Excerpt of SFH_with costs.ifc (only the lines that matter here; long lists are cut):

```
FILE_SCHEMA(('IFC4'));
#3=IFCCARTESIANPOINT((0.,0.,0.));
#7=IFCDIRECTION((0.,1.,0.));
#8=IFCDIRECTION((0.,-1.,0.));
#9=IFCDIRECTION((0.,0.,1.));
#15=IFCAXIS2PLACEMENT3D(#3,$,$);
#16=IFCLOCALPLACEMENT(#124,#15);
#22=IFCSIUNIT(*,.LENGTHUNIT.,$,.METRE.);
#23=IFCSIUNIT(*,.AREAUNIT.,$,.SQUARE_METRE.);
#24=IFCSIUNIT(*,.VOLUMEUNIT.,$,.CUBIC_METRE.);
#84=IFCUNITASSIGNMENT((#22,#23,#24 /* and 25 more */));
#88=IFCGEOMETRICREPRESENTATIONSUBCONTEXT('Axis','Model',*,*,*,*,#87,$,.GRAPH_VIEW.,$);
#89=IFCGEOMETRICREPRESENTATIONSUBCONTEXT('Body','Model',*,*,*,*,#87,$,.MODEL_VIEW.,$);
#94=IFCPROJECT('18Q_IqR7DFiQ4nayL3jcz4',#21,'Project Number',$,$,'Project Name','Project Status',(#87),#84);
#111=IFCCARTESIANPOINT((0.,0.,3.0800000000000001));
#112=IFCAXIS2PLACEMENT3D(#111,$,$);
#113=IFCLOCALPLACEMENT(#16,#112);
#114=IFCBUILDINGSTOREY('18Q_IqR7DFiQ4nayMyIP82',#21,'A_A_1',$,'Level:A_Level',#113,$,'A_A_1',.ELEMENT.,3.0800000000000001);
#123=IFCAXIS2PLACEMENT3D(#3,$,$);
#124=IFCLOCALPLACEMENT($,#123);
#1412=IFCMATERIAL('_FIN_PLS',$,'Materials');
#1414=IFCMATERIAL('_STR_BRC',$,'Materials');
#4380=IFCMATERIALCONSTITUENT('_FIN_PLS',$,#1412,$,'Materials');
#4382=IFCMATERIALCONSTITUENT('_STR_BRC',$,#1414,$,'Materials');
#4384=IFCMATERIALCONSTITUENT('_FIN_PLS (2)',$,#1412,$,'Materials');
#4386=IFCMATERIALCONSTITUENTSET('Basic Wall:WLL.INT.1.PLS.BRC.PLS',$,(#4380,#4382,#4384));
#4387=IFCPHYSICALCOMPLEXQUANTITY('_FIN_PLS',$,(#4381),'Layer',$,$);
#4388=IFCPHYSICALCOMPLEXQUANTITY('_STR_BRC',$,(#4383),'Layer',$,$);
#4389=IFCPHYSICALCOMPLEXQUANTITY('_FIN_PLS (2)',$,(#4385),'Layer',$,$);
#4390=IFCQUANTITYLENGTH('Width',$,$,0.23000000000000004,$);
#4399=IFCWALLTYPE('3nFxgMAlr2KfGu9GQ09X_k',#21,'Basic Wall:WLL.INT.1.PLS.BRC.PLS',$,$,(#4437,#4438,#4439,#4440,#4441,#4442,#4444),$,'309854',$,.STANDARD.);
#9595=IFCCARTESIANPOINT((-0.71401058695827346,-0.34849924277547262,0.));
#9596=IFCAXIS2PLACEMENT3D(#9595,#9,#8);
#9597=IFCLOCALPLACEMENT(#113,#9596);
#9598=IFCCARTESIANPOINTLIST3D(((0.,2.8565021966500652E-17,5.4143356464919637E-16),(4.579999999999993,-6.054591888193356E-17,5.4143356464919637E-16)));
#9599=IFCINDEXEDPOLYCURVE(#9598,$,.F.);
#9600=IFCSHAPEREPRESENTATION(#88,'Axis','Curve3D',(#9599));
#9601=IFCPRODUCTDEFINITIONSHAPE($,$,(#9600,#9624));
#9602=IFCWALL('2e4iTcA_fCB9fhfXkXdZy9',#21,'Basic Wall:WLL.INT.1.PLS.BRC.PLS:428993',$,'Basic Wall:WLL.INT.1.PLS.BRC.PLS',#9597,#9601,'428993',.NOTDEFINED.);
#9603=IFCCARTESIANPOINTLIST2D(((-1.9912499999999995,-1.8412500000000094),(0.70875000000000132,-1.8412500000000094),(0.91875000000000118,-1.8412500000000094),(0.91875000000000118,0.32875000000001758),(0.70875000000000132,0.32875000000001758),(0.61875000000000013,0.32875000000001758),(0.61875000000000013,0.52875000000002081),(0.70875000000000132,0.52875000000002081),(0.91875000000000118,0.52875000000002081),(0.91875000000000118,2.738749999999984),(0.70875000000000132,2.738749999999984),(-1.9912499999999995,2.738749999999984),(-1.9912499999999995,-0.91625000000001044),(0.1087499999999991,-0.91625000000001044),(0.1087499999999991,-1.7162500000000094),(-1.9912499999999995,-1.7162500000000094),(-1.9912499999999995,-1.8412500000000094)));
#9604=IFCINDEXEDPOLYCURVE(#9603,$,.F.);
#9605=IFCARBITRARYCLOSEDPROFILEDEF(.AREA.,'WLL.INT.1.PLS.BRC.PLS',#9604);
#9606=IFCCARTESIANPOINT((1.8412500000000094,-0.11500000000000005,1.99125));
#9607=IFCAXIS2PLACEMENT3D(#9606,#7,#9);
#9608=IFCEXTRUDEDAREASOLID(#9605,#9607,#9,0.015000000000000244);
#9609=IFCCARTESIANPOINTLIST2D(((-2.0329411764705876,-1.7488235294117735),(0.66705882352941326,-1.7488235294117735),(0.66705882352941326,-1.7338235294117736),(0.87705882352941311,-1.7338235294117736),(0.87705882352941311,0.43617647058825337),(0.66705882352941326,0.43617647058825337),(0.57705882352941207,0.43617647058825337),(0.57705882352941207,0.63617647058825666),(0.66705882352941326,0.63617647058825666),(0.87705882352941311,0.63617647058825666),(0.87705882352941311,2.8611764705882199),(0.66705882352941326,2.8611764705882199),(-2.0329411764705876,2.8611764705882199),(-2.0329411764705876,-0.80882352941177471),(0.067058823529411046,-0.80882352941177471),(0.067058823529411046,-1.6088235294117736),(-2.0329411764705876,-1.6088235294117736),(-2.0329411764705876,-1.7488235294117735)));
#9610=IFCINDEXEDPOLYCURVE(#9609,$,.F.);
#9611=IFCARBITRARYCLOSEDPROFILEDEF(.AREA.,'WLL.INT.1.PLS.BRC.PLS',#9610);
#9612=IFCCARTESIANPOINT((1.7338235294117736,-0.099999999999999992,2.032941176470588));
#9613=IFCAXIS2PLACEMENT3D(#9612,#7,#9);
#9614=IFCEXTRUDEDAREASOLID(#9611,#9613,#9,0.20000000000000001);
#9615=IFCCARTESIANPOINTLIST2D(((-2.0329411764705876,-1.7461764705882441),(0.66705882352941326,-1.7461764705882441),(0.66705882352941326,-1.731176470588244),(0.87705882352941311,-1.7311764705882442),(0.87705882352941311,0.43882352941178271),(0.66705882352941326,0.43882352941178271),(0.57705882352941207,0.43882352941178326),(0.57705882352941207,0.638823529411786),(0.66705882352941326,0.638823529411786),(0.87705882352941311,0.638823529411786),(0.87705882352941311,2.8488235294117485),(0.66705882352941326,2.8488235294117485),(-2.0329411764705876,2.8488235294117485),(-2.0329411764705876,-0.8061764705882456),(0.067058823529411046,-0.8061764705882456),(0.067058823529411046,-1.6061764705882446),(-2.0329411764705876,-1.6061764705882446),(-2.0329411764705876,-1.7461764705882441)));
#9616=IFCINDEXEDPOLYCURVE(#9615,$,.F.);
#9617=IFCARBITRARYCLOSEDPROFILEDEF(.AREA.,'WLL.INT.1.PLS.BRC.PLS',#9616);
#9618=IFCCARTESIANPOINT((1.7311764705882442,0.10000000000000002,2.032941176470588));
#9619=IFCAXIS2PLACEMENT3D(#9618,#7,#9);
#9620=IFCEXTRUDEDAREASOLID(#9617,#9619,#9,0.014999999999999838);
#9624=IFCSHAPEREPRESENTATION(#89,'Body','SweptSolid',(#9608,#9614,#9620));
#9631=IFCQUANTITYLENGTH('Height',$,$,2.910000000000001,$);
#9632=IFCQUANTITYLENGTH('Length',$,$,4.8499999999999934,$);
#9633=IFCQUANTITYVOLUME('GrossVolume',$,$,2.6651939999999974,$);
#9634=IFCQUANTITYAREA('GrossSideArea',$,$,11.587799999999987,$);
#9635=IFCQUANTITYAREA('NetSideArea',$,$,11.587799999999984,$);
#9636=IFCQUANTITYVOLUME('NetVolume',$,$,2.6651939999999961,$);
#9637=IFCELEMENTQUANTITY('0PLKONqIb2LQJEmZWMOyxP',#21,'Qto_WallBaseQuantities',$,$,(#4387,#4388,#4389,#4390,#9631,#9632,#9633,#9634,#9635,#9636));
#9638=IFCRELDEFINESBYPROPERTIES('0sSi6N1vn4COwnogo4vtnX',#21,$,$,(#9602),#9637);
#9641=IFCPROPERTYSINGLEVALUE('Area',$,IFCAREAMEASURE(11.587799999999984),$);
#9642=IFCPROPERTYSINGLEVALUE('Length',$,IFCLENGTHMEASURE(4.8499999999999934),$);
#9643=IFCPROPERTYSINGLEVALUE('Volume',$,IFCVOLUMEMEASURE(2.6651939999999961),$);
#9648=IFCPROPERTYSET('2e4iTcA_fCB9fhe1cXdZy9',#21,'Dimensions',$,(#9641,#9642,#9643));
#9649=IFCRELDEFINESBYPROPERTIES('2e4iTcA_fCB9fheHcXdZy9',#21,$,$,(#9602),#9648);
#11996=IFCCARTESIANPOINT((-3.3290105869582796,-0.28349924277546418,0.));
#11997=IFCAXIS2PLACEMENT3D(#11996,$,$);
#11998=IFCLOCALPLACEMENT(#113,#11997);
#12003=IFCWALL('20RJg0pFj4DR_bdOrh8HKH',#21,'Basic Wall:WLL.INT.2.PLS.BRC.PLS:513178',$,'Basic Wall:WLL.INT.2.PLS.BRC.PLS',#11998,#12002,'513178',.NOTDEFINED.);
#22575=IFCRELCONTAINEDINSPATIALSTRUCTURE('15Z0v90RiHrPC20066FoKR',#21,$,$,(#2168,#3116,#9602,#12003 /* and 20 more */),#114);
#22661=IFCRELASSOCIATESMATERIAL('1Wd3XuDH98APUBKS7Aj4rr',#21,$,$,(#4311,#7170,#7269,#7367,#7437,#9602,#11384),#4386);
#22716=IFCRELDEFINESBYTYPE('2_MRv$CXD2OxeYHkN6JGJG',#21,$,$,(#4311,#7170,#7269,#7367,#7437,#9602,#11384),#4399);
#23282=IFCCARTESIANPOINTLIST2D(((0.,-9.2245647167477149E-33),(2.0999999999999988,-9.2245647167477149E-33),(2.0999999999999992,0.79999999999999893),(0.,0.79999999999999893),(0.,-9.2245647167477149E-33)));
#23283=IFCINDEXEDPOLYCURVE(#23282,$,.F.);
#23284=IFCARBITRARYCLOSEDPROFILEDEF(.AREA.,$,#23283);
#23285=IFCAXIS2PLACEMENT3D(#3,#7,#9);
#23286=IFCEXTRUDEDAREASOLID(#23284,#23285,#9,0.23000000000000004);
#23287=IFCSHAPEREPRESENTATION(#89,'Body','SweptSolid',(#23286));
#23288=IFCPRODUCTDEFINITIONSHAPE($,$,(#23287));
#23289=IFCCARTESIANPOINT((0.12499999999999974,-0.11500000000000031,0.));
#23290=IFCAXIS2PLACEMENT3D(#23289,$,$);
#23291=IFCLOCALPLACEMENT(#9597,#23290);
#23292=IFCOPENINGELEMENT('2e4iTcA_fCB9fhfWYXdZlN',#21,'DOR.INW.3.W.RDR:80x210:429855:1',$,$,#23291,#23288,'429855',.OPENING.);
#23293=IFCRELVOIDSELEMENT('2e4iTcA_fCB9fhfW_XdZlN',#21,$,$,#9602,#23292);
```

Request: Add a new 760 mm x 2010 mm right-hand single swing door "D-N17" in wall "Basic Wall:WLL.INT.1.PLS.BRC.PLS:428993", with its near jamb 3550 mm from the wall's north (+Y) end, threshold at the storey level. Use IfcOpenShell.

```python
import numpy as np
import ifcopenshell
import ifcopenshell.api.feature
import ifcopenshell.api.geometry
import ifcopenshell.api.pset
import ifcopenshell.api.root
import ifcopenshell.api.spatial
import ifcopenshell.geom
import ifcopenshell.util.element
import ifcopenshell.util.placement
import ifcopenshell.util.representation
import ifcopenshell.util.shape
import ifcopenshell.util.unit

model = ifcopenshell.open("SFH_with costs.ifc")
unit_scale = ifcopenshell.util.unit.calculate_unit_scale(model)
area_scale = ifcopenshell.util.unit.calculate_unit_scale(model, "AREAUNIT")
volume_scale = ifcopenshell.util.unit.calculate_unit_scale(model, "VOLUMEUNIT")
settings = ifcopenshell.geom.settings()


def volume(element):
    """Net volume in cubic metres, openings subtracted."""
    shape = ifcopenshell.geom.create_shape(settings, element)
    return ifcopenshell.util.shape.get_volume(shape.geometry)


wall = model.by_guid("2e4iTcA_fCB9fhfXkXdZy9")
storey = ifcopenshell.util.element.get_container(wall, ifc_class="IfcBuildingStorey")
context = ifcopenshell.util.representation.get_context(model, "Model", "Body", "MODEL_VIEW")
before = volume(wall)

width, height, from_end, sill = 0.76, 2.01, 3.55, 0.0  # metres

# The wall runs along its own X axis, and the end named is its -X end.
wall_shape = ifcopenshell.geom.create_shape(settings, wall)
x, y, z = ifcopenshell.util.shape.get_vertices(wall_shape.geometry).T
start = x.min() + from_end
face, thickness = float(y.min()), float(y.max() - y.min())
wall_matrix = ifcopenshell.util.placement.get_local_placement(wall.ObjectPlacement)
level = ifcopenshell.util.placement.get_local_placement(storey.ObjectPlacement)[2, 3]


def in_wall(x, y):
    """Placement at x, y metres in the wall's axes, at sill height."""
    matrix = wall_matrix.copy()
    matrix[:, 3] = wall_matrix @ np.array([x / unit_scale, y / unit_scale, 0.0, 1.0])
    matrix[2, 3] = level + sill / unit_scale
    return matrix


# Opening: a box that overshoots both wall faces by 50 mm.
opening = ifcopenshell.api.root.create_entity(model, ifc_class="IfcOpeningElement", predefined_type="OPENING")
box = ifcopenshell.api.geometry.add_wall_representation(
    model, context=context, length=width, height=height, thickness=thickness + 0.1
)
ifcopenshell.api.geometry.assign_representation(model, product=opening, representation=box)
ifcopenshell.api.geometry.edit_object_placement(model, product=opening, matrix=in_wall(start, face - 0.05), is_si=False)
ifcopenshell.api.feature.add_feature(model, feature=opening, element=wall)

door = ifcopenshell.api.root.create_entity(model, ifc_class="IfcDoor", name="D-N17", predefined_type="DOOR")
door.OverallWidth, door.OverallHeight = width / unit_scale, height / unit_scale
door.OperationType = "SINGLE_SWING_RIGHT"
body = ifcopenshell.api.geometry.add_door_representation(
    model,
    context=context,
    overall_width=door.OverallWidth,
    overall_height=door.OverallHeight,
    operation_type="SINGLE_SWING_RIGHT",
    lining_properties={"LiningDepth": thickness / unit_scale, "ThresholdDepth": thickness / unit_scale},
)
ifcopenshell.api.geometry.assign_representation(model, product=door, representation=body)
ifcopenshell.api.spatial.assign_container(model, products=[door], relating_structure=storey)
ifcopenshell.api.feature.add_filling(model, opening=opening, element=door)

# The lining spans the wall, so the door starts at the wall face.
ifcopenshell.api.geometry.edit_object_placement(model, product=door, matrix=in_wall(start, face), is_si=False)

after = volume(wall)

# Update the wall's stored quantities.
qto = model.by_id(ifcopenshell.util.element.get_pset(wall, "Qto_WallBaseQuantities", should_inherit=False)["id"])
ifcopenshell.api.pset.edit_qto(model, qto=qto, properties={
    "NetSideArea": after / thickness / area_scale,
    "NetVolume": after / volume_scale,
})
pset = model.by_id(ifcopenshell.util.element.get_pset(wall, "Dimensions", should_inherit=False)["id"])
ifcopenshell.api.pset.edit_pset(model, pset=pset, properties={
    "Area": model.create_entity("IfcAreaMeasure", after / thickness / area_scale),
    "Volume": model.create_entity("IfcVolumeMeasure", after / volume_scale),
})

print(f"wall volume {before:.3f} -> {after:.3f} m3")

model.write("SFH_with costs-out.ifc")
```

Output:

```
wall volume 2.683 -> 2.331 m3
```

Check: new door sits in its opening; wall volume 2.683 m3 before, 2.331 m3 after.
